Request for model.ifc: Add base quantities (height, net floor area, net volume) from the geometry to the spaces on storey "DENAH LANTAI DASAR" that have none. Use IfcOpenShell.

First a look at what the model holds.

```python
import ifcopenshell
import ifcopenshell.util.element
import ifcopenshell.util.unit

model = ifcopenshell.open("model.ifc")
print(model.schema)
for unit_type in ("LENGTHUNIT", "AREAUNIT", "VOLUMEUNIT"):
    print(unit_type, ifcopenshell.util.unit.calculate_unit_scale(model, unit_type))
storey = next(s for s in model.by_type("IfcBuildingStorey") if s.Name == "DENAH LANTAI DASAR")
spaces = [e for e in ifcopenshell.util.element.get_decomposition(storey) if e.is_a("IfcSpace")]
for e in sorted(spaces, key=lambda e: e.id()):
    print(e.id(), e.is_a(), e.Name, list(ifcopenshell.util.element.get_psets(e, qtos_only=True)), sep=" | ")
```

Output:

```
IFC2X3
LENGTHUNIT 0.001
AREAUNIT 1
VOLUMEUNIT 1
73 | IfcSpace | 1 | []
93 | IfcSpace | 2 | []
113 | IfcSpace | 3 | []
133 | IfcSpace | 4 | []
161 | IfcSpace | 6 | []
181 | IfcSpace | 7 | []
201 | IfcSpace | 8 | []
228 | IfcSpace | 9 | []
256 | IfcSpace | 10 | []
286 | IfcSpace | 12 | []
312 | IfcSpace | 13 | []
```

```python
import ifcopenshell
import ifcopenshell.api.pset
import ifcopenshell.geom
import ifcopenshell.util.element
import ifcopenshell.util.shape
import ifcopenshell.util.unit

model = ifcopenshell.open("model.ifc")
unit_scale = ifcopenshell.util.unit.calculate_unit_scale(model)
area_scale = ifcopenshell.util.unit.calculate_unit_scale(model, "AREAUNIT")
volume_scale = ifcopenshell.util.unit.calculate_unit_scale(model, "VOLUMEUNIT")
settings = ifcopenshell.geom.settings()

storey = next(s for s in model.by_type("IfcBuildingStorey") if s.Name == "DENAH LANTAI DASAR")
spaces = [e for e in ifcopenshell.util.element.get_decomposition(storey) if e.is_a("IfcSpace")]

for e in sorted(spaces, key=lambda e: e.id()):
    if ifcopenshell.util.element.get_psets(e, qtos_only=True, should_inherit=False):
        continue
    # Geometry comes back in metres, in the element's own axes.
    shape = ifcopenshell.geom.create_shape(settings, e)
    values = {
        "Height": ifcopenshell.util.shape.get_z(shape.geometry) / unit_scale,
        "NetFloorArea": ifcopenshell.util.shape.get_footprint_area(shape.geometry) / area_scale,
        "NetVolume": ifcopenshell.util.shape.get_volume(shape.geometry) / volume_scale,
    }
    qto = ifcopenshell.api.pset.add_qto(model, product=e, name="BaseQuantities")
    ifcopenshell.api.pset.edit_qto(model, qto=qto, properties=values)
    print(e.id(), {k: round(v, 3) for k, v in values.items()})

model.write("model_v2.ifc")
```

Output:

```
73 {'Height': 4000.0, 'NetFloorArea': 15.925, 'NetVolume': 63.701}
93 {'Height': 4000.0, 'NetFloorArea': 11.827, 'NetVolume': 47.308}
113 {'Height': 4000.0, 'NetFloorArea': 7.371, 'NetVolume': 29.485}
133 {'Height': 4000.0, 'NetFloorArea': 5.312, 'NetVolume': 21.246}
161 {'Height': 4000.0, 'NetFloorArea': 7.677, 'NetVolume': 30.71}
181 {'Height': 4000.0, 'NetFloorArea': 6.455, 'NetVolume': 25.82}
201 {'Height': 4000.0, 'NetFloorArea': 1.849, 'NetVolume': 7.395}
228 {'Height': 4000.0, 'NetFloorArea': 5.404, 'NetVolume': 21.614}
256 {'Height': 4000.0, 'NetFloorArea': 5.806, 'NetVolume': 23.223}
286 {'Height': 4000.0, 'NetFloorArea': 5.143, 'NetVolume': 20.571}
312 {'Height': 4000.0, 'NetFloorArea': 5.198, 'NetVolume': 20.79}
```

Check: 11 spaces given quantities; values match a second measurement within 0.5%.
